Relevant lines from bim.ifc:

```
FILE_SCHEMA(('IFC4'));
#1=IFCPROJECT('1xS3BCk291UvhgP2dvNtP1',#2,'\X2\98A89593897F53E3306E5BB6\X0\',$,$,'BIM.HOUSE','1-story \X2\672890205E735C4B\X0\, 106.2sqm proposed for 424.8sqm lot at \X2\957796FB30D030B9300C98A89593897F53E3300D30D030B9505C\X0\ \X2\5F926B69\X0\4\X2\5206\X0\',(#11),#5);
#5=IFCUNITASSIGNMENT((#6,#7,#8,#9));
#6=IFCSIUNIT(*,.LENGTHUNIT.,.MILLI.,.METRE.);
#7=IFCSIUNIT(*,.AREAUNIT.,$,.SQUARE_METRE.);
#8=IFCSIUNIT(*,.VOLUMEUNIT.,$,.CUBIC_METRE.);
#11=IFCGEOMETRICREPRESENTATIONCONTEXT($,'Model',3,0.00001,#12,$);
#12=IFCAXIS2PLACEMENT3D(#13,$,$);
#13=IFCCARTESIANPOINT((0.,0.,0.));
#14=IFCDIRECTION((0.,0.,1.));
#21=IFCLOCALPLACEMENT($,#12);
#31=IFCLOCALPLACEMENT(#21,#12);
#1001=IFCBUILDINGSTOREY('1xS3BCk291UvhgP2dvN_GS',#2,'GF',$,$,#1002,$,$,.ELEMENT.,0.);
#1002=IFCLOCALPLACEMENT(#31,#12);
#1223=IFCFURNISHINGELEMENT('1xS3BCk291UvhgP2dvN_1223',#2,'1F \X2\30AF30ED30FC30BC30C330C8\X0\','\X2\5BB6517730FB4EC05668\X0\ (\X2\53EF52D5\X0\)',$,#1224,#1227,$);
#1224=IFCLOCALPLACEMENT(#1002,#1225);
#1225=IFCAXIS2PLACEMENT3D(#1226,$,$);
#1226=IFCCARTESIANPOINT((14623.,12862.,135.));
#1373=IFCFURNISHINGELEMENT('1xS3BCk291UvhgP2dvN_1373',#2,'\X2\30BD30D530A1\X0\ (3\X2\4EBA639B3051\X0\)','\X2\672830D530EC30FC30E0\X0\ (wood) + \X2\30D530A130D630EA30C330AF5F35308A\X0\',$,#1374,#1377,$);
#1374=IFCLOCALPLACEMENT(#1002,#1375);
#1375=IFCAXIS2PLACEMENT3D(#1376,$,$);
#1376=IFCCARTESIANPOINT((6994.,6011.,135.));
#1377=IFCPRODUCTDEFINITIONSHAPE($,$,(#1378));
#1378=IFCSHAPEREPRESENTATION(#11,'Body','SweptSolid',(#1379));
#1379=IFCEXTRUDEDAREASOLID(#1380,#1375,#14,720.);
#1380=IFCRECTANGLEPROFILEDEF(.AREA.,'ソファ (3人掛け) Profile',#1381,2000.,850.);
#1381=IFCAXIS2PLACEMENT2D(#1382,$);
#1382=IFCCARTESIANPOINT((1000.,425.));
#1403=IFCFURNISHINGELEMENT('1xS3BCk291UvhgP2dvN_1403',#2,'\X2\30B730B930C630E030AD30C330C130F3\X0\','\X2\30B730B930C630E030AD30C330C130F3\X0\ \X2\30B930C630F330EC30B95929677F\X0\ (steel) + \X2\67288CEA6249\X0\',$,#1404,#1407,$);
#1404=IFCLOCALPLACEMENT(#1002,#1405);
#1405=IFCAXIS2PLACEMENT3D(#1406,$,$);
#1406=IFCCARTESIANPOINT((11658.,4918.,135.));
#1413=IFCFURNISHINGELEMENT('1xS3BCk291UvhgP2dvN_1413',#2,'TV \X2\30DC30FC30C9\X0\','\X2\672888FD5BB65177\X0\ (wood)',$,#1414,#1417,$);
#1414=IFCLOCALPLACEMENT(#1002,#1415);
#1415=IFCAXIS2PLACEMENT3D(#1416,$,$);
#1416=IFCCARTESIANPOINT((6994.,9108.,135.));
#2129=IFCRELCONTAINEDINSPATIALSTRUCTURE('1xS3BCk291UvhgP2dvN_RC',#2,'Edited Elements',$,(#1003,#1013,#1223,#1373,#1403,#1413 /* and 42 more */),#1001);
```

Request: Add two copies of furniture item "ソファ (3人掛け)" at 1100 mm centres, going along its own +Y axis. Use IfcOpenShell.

```python
import ifcopenshell
import ifcopenshell.api.geometry
import ifcopenshell.api.root
import ifcopenshell.util.element
import ifcopenshell.util.placement
import ifcopenshell.util.unit

model = ifcopenshell.open("bim.ifc")
unit_scale = ifcopenshell.util.unit.calculate_unit_scale(model)


def reuse_history(source, copy):
    """copy_class also copies each property set's owner history, people and application; keep the originals."""
    for rel in copy.IsDefinedBy:
        if rel.is_a("IfcRelDefinesByProperties") and (history := rel.RelatingPropertyDefinition.OwnerHistory):
            rel.RelatingPropertyDefinition.OwnerHistory = source.OwnerHistory
            ifcopenshell.util.element.remove_deep2(model, history)


source = model.by_guid("1xS3BCk291UvhgP2dvN_1373")
base = ifcopenshell.util.placement.get_local_placement(source.ObjectPlacement)
step = base[:3, 1] * 1.1 / unit_scale

for i in range(1, 3):
    copy = ifcopenshell.api.root.copy_class(model, product=source)
    copy.Representation = ifcopenshell.util.element.copy_deep(
        model, source.Representation, exclude=["IfcGeometricRepresentationContext", "IfcRepresentationMap"]
    )
    reuse_history(source, copy)
    matrix = base.copy()
    matrix[:3, 3] += i * step
    print("added at", matrix[:3, 3].round(3) + 0.0)
    ifcopenshell.api.geometry.edit_object_placement(model, product=copy, matrix=matrix, is_si=False)

model.write("bim_rev.ifc")
```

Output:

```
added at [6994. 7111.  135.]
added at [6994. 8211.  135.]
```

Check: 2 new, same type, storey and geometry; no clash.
